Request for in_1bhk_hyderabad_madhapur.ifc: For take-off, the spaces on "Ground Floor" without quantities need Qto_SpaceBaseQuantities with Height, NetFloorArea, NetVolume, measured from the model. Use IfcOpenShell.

First a look at what the model holds.

```python
import ifcopenshell
import ifcopenshell.util.element
import ifcopenshell.util.unit

model = ifcopenshell.open("in_1bhk_hyderabad_madhapur.ifc")
print(model.schema)
for unit_type in ("LENGTHUNIT", "AREAUNIT", "VOLUMEUNIT"):
    print(unit_type, ifcopenshell.util.unit.calculate_unit_scale(model, unit_type))
storey = next(s for s in model.by_type("IfcBuildingStorey") if s.Name == "Ground Floor")
spaces = [e for e in ifcopenshell.util.element.get_decomposition(storey) if e.is_a("IfcSpace")]
for e in sorted(spaces, key=lambda e: e.id()):
    print(e.id(), e.is_a(), e.Name, list(ifcopenshell.util.element.get_psets(e, qtos_only=True)), sep=" | ")
```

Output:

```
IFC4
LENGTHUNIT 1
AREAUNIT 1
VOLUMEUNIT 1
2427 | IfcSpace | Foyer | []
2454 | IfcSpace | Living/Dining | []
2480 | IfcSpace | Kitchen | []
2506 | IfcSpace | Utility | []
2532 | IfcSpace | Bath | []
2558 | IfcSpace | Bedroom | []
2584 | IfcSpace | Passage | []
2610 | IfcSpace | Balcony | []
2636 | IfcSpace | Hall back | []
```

```python
import ifcopenshell
import ifcopenshell.api.pset
import ifcopenshell.geom
import ifcopenshell.util.element
import ifcopenshell.util.shape
import ifcopenshell.util.unit

model = ifcopenshell.open("in_1bhk_hyderabad_madhapur.ifc")
unit_scale = ifcopenshell.util.unit.calculate_unit_scale(model)
area_scale = ifcopenshell.util.unit.calculate_unit_scale(model, "AREAUNIT")
volume_scale = ifcopenshell.util.unit.calculate_unit_scale(model, "VOLUMEUNIT")
settings = ifcopenshell.geom.settings()

storey = next(s for s in model.by_type("IfcBuildingStorey") if s.Name == "Ground Floor")
spaces = [e for e in ifcopenshell.util.element.get_decomposition(storey) if e.is_a("IfcSpace")]

for e in sorted(spaces, key=lambda e: e.id()):
    if ifcopenshell.util.element.get_psets(e, qtos_only=True, should_inherit=False):
        continue
    # Geometry comes back in metres, in the element's own axes.
    shape = ifcopenshell.geom.create_shape(settings, e)
    values = {
        "Height": ifcopenshell.util.shape.get_z(shape.geometry) / unit_scale,
        "NetFloorArea": ifcopenshell.util.shape.get_footprint_area(shape.geometry) / area_scale,
        "NetVolume": ifcopenshell.util.shape.get_volume(shape.geometry) / volume_scale,
    }
    qto = ifcopenshell.api.pset.add_qto(model, product=e, name="Qto_SpaceBaseQuantities")
    ifcopenshell.api.pset.edit_qto(model, qto=qto, properties=values)
    print(e.id(), {k: round(v, 3) for k, v in values.items()})

model.write("in_1bhk_hyderabad_madhapur_v2.ifc")
```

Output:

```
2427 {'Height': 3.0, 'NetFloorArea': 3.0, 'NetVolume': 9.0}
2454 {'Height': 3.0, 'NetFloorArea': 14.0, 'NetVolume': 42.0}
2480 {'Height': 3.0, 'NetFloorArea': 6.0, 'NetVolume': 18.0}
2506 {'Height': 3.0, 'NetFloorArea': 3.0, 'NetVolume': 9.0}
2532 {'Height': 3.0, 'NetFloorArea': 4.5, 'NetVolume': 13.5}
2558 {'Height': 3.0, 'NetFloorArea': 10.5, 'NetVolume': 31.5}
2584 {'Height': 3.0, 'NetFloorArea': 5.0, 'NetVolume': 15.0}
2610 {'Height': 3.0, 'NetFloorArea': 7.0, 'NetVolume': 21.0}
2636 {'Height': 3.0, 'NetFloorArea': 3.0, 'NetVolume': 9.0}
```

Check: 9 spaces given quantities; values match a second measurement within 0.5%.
